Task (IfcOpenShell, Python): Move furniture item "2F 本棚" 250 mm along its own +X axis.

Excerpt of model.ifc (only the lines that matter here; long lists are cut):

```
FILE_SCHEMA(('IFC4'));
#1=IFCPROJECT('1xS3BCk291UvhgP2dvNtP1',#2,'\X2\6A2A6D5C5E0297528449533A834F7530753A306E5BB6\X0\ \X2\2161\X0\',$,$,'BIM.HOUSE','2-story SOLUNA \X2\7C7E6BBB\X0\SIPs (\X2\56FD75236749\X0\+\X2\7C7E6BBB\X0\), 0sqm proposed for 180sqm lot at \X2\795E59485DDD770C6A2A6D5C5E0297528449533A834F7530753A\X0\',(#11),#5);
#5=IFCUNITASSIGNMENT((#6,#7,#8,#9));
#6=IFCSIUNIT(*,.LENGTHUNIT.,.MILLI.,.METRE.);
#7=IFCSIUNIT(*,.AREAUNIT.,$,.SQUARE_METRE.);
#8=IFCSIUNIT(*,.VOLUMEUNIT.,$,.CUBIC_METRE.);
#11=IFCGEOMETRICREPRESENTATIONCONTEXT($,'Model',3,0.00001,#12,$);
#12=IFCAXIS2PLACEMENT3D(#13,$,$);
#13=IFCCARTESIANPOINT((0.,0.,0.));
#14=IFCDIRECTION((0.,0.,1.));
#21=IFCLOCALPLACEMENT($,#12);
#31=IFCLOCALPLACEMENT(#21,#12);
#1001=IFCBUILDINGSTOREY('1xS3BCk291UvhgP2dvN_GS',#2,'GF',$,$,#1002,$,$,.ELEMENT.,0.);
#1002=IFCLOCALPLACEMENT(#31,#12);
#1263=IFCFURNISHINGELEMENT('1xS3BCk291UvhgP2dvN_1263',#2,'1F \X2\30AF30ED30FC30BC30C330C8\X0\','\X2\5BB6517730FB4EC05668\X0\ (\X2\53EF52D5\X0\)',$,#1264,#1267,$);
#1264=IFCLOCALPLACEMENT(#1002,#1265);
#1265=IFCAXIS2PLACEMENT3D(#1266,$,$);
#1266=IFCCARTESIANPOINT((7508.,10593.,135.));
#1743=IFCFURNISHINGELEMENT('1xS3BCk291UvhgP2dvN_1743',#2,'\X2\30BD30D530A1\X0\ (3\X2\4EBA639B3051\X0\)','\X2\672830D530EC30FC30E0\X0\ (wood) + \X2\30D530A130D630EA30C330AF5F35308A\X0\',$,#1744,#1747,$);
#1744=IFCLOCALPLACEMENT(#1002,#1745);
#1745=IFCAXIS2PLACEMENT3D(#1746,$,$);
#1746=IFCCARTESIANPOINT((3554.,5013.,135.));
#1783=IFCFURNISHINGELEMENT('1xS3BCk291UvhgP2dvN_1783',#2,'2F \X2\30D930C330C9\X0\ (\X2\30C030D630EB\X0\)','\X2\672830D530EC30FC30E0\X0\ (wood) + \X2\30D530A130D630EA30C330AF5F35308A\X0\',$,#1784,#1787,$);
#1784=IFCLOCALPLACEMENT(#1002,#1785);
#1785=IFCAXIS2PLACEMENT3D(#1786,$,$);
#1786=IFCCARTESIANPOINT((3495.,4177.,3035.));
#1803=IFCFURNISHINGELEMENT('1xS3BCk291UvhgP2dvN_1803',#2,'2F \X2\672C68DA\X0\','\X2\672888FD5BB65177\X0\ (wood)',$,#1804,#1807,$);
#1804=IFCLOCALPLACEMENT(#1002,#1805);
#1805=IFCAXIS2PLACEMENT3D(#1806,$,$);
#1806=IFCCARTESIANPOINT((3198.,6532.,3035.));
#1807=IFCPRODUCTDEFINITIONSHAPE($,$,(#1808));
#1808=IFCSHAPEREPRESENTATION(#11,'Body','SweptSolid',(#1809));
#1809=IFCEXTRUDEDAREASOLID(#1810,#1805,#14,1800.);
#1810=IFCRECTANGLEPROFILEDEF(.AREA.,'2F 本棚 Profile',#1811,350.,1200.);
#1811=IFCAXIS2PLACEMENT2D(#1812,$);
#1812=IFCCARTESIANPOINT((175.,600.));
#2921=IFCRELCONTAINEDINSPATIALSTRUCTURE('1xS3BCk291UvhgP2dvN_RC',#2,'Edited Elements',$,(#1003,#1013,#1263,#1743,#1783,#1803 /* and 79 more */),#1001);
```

```python
import ifcopenshell
import ifcopenshell.api.geometry
import ifcopenshell.util.placement
import ifcopenshell.util.unit

model = ifcopenshell.open("model.ifc")
unit_scale = ifcopenshell.util.unit.calculate_unit_scale(model)

item = model.by_guid("1xS3BCk291UvhgP2dvN_1803")
matrix = ifcopenshell.util.placement.get_local_placement(item.ObjectPlacement)
matrix[:3, 3] += matrix[:3, 0] * 0.25 / unit_scale
ifcopenshell.api.geometry.edit_object_placement(model, product=item, matrix=matrix, is_si=False)

print(ifcopenshell.util.placement.get_local_placement(item.ObjectPlacement).round(3) + 0.0)

model.write("model_edited.ifc")
```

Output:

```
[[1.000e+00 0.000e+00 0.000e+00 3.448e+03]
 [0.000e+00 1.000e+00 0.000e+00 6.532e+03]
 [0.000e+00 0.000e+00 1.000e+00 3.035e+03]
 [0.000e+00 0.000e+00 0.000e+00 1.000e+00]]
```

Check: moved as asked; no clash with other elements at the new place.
